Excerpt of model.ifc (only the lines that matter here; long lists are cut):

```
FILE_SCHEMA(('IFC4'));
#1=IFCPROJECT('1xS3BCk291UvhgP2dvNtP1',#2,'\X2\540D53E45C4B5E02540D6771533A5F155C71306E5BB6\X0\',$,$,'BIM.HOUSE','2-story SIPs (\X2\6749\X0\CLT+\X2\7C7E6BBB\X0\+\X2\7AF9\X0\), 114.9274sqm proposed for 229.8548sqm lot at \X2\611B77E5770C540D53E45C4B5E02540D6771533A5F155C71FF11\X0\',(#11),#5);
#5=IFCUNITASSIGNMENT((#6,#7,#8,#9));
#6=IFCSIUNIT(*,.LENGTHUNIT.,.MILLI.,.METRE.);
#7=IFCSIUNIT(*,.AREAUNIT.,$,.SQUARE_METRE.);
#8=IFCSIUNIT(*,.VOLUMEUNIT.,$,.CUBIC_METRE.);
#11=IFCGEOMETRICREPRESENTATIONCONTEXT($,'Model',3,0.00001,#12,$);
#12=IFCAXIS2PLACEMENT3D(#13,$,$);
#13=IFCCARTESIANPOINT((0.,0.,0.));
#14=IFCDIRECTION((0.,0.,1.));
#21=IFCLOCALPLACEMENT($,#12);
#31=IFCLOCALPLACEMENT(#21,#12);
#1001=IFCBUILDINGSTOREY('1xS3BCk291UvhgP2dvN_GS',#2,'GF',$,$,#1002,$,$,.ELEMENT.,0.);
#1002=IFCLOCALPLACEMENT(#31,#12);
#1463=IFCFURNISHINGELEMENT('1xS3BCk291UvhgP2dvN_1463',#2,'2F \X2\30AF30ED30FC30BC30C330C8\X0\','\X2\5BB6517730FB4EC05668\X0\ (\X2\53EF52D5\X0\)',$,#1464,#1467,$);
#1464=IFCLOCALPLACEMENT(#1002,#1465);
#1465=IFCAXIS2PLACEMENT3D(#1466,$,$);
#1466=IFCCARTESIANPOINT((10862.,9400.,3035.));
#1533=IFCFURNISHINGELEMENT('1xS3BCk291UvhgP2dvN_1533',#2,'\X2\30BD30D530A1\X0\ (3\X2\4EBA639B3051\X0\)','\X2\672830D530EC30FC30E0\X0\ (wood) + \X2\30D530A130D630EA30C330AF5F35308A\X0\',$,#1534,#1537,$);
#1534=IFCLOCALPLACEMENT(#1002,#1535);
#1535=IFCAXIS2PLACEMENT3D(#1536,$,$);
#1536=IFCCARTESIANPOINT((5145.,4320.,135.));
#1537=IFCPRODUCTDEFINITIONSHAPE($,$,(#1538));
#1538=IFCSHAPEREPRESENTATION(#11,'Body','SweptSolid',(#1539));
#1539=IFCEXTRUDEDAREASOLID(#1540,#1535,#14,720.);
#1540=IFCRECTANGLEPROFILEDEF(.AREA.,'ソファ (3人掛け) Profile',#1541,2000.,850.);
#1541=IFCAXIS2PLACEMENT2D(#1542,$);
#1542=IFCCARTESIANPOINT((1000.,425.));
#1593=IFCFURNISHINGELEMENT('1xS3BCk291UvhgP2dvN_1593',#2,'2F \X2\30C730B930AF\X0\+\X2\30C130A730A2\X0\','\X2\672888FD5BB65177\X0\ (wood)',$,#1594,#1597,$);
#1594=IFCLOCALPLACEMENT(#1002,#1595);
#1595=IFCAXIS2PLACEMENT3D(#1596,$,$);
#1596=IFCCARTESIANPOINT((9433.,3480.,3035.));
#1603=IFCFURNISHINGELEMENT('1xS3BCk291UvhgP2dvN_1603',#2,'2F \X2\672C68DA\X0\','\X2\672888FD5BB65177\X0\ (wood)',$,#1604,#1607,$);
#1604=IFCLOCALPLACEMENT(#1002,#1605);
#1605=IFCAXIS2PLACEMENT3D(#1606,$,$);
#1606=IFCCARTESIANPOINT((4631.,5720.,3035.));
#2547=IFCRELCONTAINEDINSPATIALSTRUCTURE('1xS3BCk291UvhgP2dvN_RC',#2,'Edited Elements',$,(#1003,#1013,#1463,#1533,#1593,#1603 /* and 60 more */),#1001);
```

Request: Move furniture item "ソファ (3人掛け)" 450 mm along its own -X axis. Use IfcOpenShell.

```python
import ifcopenshell
import ifcopenshell.api.geometry
import ifcopenshell.util.placement

model = ifcopenshell.open("model.ifc")

item = model.by_guid("1xS3BCk291UvhgP2dvN_1533")
matrix = ifcopenshell.util.placement.get_local_placement(item.ObjectPlacement)
matrix[:3, 3] -= matrix[:3, 0] * 450.0
ifcopenshell.api.geometry.edit_object_placement(model, product=item, matrix=matrix, is_si=False)

print(ifcopenshell.util.placement.get_local_placement(item.ObjectPlacement).round(3) + 0.0)

model.write("model_v2.ifc")
```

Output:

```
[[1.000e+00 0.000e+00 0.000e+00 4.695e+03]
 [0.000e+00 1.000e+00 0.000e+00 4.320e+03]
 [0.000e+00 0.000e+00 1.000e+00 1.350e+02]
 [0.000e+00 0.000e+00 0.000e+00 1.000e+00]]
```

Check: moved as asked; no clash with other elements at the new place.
